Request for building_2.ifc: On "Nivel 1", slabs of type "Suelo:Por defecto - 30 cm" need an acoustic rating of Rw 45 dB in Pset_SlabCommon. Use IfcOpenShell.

First a look at what the model holds.

```python
import ifcopenshell
import ifcopenshell.util.element

model = ifcopenshell.open("building_2.ifc")
print(model.schema)
storey = next(s for s in model.by_type("IfcBuildingStorey") if s.Name == "Nivel 1")
slabs = [e for e in ifcopenshell.util.element.get_decomposition(storey) if e.is_a("IfcSlab")]
seen = {}
for e in slabs:
    element_type = ifcopenshell.util.element.get_type(e)
    key = (element_type.Name if element_type != e and element_type else None, ifcopenshell.util.element.get_pset(e, "Pset_SlabCommon", "AcousticRating"))
    seen[key] = seen.get(key, 0) + 1
for (name, value), count in sorted(seen.items(), key=str):
    print(count, "x", name, "|", value)
```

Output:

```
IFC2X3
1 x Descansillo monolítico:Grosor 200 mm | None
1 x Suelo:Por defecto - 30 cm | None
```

```python
import ifcopenshell
import ifcopenshell.api.pset
import ifcopenshell.util.element

model = ifcopenshell.open("building_2.ifc")

storey = next(s for s in model.by_type("IfcBuildingStorey") if s.Name == "Nivel 1")
slabs = [e for e in ifcopenshell.util.element.get_decomposition(storey) if e.is_a("IfcSlab")]

count = 0
for e in slabs:
    element_type = ifcopenshell.util.element.get_type(e)
    if element_type in (None, e) or element_type.Name != "Suelo:Por defecto - 30 cm":
        continue
    # add_pset returns the element's existing set when there is one.
    pset = ifcopenshell.api.pset.add_pset(model, product=e, name="Pset_SlabCommon")
    ifcopenshell.api.pset.edit_pset(model, pset=pset, properties={"AcousticRating": "Rw 45 dB"})
    count += 1

print(count, "slabs updated")

model.write("building_2_rev.ifc")
```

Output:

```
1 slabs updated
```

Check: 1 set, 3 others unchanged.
